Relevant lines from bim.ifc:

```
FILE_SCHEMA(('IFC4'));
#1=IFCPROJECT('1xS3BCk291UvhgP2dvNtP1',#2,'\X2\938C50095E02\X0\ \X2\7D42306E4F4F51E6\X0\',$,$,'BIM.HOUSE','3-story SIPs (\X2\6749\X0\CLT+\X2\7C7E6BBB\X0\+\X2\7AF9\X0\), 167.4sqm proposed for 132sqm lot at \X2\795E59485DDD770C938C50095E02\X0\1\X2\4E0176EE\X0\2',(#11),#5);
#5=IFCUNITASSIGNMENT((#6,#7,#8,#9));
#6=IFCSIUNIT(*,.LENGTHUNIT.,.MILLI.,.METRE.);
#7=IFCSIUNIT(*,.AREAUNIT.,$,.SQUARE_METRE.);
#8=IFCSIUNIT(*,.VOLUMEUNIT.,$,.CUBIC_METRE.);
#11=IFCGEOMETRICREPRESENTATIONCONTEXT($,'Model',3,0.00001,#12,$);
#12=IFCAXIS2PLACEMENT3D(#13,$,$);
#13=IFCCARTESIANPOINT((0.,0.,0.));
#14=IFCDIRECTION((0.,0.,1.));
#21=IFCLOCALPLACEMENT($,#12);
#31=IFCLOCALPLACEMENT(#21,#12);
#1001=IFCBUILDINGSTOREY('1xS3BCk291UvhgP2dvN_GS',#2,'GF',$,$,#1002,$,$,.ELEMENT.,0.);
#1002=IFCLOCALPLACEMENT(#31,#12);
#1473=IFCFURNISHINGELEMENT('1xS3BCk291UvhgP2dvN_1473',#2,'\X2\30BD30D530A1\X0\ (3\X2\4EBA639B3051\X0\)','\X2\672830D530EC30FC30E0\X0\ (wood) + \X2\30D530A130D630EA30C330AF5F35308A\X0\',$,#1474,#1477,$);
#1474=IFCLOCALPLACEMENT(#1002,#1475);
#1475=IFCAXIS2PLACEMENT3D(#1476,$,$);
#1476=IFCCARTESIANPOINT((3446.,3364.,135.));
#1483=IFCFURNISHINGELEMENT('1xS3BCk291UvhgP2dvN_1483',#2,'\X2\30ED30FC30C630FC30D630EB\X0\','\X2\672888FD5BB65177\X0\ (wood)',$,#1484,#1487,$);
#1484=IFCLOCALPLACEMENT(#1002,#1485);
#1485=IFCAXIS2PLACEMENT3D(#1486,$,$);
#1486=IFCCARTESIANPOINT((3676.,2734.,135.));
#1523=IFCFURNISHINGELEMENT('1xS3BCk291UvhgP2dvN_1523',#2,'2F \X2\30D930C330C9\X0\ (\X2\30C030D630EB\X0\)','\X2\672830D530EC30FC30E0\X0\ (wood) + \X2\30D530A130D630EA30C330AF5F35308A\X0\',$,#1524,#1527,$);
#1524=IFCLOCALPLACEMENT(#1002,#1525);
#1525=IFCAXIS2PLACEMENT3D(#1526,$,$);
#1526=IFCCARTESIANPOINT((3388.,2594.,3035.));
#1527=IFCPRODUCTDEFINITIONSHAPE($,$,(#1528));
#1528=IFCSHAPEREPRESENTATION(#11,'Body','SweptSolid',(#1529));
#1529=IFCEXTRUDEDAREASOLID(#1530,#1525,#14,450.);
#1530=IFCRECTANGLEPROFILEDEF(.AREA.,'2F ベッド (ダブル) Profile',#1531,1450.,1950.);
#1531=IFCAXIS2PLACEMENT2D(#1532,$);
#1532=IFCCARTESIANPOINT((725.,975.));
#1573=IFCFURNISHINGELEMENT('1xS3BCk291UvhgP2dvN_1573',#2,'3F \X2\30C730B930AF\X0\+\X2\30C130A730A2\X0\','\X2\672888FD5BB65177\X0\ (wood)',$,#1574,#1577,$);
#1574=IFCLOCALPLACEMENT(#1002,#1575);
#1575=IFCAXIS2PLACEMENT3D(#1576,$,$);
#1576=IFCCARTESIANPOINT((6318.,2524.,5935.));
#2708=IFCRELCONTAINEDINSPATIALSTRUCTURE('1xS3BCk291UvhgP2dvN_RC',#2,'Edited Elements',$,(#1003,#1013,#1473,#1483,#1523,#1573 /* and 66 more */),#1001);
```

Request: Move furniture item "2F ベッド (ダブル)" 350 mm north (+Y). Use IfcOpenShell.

```python
import ifcopenshell
import ifcopenshell.api.geometry
import ifcopenshell.util.placement
import ifcopenshell.util.unit

model = ifcopenshell.open("bim.ifc")
unit_scale = ifcopenshell.util.unit.calculate_unit_scale(model)

item = model.by_id(1523)
matrix = ifcopenshell.util.placement.get_local_placement(item.ObjectPlacement)
matrix[1, 3] += 0.35 / unit_scale
ifcopenshell.api.geometry.edit_object_placement(model, product=item, matrix=matrix, is_si=False)

print(ifcopenshell.util.placement.get_local_placement(item.ObjectPlacement).round(3) + 0.0)

model.write("bim_v2.ifc")
```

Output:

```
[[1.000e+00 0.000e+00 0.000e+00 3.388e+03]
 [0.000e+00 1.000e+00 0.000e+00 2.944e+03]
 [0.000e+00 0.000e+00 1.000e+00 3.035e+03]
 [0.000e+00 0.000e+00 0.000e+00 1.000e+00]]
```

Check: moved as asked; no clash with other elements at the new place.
